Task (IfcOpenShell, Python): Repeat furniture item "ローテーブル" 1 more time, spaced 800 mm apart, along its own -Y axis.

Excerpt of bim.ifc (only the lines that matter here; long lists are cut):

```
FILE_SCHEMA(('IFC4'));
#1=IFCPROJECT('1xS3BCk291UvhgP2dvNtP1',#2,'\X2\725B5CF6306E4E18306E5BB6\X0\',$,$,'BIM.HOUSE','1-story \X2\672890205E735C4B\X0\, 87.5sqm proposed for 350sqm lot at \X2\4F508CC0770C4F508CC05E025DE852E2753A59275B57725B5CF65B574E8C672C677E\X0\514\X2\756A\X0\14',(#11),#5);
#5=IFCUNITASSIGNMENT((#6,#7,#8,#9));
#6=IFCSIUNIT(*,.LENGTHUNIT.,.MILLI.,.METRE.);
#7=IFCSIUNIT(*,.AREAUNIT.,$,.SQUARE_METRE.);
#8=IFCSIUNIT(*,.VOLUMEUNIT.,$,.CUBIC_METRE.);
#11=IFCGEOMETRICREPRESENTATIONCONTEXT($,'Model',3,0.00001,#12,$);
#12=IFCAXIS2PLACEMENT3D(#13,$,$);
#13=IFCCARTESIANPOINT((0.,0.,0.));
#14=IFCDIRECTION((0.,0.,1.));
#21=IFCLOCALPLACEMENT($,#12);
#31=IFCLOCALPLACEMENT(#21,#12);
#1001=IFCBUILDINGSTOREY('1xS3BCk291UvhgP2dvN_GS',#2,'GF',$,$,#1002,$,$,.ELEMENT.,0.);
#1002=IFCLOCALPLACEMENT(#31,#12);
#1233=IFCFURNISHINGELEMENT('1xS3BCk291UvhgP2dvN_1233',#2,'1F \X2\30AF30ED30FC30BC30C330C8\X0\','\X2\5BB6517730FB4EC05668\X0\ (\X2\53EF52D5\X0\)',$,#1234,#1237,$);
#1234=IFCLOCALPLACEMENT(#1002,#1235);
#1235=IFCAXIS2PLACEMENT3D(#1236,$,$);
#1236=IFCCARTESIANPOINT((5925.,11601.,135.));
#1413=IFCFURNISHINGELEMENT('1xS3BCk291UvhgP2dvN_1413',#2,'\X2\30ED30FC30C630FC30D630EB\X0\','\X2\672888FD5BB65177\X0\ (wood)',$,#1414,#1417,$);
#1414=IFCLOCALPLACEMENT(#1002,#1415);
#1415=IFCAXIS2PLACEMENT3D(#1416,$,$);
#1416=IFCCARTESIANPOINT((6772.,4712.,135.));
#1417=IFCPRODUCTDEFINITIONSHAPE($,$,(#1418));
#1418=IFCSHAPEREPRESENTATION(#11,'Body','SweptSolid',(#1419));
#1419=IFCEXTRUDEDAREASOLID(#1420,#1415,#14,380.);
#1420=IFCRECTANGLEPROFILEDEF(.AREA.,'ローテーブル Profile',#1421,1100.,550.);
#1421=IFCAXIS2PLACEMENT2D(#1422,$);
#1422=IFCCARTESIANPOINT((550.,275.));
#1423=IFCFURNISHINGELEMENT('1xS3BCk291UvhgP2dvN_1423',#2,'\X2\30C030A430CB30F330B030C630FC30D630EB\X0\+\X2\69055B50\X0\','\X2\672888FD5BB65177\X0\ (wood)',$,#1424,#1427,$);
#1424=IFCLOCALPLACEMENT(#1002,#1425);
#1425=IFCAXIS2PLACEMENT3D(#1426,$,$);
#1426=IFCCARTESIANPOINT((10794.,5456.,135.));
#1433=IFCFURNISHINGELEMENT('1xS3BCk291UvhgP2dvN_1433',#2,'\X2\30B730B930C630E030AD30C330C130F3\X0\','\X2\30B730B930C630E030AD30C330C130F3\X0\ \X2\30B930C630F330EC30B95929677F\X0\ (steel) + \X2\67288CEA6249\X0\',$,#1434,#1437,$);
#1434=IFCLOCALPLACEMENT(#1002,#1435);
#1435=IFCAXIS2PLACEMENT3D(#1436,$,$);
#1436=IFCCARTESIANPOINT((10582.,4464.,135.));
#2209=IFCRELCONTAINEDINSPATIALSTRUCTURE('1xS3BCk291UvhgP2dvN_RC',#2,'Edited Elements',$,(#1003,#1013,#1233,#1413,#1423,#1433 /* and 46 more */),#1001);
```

```python
import ifcopenshell
import ifcopenshell.api.geometry
import ifcopenshell.api.root
import ifcopenshell.util.element
import ifcopenshell.util.placement
import ifcopenshell.util.unit

model = ifcopenshell.open("bim.ifc")
unit_scale = ifcopenshell.util.unit.calculate_unit_scale(model)


def reuse_history(source, copy):
    """copy_class also copies each property set's owner history, people and application; keep the originals."""
    for rel in copy.IsDefinedBy:
        if rel.is_a("IfcRelDefinesByProperties") and (history := rel.RelatingPropertyDefinition.OwnerHistory):
            rel.RelatingPropertyDefinition.OwnerHistory = source.OwnerHistory
            ifcopenshell.util.element.remove_deep2(model, history)


source = model.by_guid("1xS3BCk291UvhgP2dvN_1413")
base = ifcopenshell.util.placement.get_local_placement(source.ObjectPlacement)
step = -base[:3, 1] * 0.8 / unit_scale

for i in range(1, 2):
    copy = ifcopenshell.api.root.copy_class(model, product=source)
    copy.Representation = ifcopenshell.util.element.copy_deep(
        model, source.Representation, exclude=["IfcGeometricRepresentationContext", "IfcRepresentationMap"]
    )
    reuse_history(source, copy)
    matrix = base.copy()
    matrix[:3, 3] += i * step
    print("added at", matrix[:3, 3].round(3) + 0.0)
    ifcopenshell.api.geometry.edit_object_placement(model, product=copy, matrix=matrix, is_si=False)

model.write("bim-out.ifc")
```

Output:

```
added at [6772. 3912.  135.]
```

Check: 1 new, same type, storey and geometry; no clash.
